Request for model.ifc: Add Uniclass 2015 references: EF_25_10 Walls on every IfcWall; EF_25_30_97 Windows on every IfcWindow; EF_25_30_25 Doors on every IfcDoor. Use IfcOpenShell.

First a look at what the model holds.

```python
import ifcopenshell

model = ifcopenshell.open("model.ifc")
print(model.schema)
print("classifications:", [c.Name for c in model.by_type("IfcClassification")])
for ifc_class in ("IfcDoor", "IfcRoof", "IfcStair", "IfcWall", "IfcWindow"):
    print(ifc_class, len(model.by_type(ifc_class)))
```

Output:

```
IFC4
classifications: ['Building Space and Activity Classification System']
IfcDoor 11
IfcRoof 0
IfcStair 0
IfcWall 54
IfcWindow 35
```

```python
import ifcopenshell
import ifcopenshell.api.classification

model = ifcopenshell.open("model.ifc")

system = ifcopenshell.api.classification.add_classification(model, classification="Uniclass 2015")

codes = {
    "IfcWall": ("EF_25_10", "Walls"),
    "IfcWindow": ("EF_25_30_97", "Windows"),
    "IfcDoor": ("EF_25_30_25", "Doors"),
}
for ifc_class, (code, name) in codes.items():
    products = model.by_type(ifc_class)
    ifcopenshell.api.classification.add_reference(
        model, products=products, classification=system, identification=code, name=name
    )
    print(code, len(products))

model.write("model_edited.ifc")
```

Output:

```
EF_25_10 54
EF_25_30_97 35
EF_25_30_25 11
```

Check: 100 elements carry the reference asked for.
